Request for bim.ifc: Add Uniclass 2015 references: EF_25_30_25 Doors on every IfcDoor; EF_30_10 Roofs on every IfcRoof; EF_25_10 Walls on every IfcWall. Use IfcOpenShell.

First a look at what the model holds.

```python
import ifcopenshell

model = ifcopenshell.open("bim.ifc")
print(model.schema)
print("classifications:", [c.Name for c in model.by_type("IfcClassification")])
for ifc_class in ("IfcDoor", "IfcRoof", "IfcStair", "IfcWall", "IfcWindow"):
    print(ifc_class, len(model.by_type(ifc_class)))
```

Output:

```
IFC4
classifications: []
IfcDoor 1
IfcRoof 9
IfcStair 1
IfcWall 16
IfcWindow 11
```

```python
import ifcopenshell
import ifcopenshell.api.classification

model = ifcopenshell.open("bim.ifc")

system = ifcopenshell.api.classification.add_classification(model, classification="Uniclass 2015")

codes = {
    "IfcDoor": ("EF_25_30_25", "Doors"),
    "IfcRoof": ("EF_30_10", "Roofs"),
    "IfcWall": ("EF_25_10", "Walls"),
}
for ifc_class, (code, name) in codes.items():
    products = model.by_type(ifc_class)
    ifcopenshell.api.classification.add_reference(
        model, products=products, classification=system, identification=code, name=name
    )
    print(code, len(products))

model.write("bim_updated.ifc")
```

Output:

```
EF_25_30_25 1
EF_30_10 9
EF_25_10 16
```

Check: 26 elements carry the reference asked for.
